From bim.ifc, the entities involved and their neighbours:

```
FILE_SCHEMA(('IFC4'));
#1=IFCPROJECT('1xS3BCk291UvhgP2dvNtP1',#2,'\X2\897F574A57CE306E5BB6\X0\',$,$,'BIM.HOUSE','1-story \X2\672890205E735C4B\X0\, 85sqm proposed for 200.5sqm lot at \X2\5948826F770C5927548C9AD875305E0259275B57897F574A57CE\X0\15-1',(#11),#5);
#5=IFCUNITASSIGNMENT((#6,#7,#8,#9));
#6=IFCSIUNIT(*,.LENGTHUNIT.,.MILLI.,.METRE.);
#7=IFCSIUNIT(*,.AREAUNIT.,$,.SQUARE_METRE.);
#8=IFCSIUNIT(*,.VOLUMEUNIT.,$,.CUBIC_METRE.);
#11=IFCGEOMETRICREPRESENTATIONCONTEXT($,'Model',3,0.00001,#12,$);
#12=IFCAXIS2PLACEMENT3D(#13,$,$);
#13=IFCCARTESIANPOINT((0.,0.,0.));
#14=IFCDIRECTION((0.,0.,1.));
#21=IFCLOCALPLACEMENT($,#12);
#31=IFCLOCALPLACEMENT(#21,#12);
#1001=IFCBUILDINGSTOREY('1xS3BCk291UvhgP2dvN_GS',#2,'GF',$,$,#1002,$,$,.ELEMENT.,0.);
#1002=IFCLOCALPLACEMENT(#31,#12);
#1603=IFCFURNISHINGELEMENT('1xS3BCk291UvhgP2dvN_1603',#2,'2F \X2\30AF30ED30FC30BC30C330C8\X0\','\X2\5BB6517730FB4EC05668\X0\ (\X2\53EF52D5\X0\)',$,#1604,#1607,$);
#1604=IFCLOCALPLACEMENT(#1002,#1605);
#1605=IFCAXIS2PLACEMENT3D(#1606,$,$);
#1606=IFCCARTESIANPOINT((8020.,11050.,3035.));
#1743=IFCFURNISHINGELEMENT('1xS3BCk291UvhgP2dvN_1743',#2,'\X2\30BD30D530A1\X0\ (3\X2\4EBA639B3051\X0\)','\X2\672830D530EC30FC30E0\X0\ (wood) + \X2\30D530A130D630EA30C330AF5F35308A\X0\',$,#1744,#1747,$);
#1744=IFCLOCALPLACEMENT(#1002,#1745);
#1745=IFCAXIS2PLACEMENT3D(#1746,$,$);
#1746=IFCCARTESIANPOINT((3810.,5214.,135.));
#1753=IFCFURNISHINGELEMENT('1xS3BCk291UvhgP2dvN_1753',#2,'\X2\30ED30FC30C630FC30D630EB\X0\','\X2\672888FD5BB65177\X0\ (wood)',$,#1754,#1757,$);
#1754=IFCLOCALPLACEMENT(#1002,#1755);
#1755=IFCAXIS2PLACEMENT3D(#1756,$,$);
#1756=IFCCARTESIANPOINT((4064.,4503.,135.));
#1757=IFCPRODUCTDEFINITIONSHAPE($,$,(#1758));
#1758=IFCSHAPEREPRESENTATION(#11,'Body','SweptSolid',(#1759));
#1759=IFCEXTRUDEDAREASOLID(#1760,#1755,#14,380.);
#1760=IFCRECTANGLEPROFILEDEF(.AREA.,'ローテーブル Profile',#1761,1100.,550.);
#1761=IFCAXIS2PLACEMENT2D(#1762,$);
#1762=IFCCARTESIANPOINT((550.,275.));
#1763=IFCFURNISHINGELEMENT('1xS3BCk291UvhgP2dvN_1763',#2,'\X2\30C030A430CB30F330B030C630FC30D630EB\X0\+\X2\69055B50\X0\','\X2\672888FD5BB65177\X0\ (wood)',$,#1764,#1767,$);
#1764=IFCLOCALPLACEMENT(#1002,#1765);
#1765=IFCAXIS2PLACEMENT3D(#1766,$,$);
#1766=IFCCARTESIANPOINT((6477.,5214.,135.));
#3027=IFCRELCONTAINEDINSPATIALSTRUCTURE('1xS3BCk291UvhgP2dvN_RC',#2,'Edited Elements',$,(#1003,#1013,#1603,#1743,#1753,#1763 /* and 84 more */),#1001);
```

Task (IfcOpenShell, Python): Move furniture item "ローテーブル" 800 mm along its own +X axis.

```python
import ifcopenshell
import ifcopenshell.api.geometry
import ifcopenshell.util.placement
import ifcopenshell.util.unit

model = ifcopenshell.open("bim.ifc")
unit_scale = ifcopenshell.util.unit.calculate_unit_scale(model)

item = model.by_id(1753)
matrix = ifcopenshell.util.placement.get_local_placement(item.ObjectPlacement)
matrix[:3, 3] += matrix[:3, 0] * 0.8 / unit_scale
ifcopenshell.api.geometry.edit_object_placement(model, product=item, matrix=matrix, is_si=False)

print(ifcopenshell.util.placement.get_local_placement(item.ObjectPlacement).round(3) + 0.0)

model.write("bim-out.ifc")
```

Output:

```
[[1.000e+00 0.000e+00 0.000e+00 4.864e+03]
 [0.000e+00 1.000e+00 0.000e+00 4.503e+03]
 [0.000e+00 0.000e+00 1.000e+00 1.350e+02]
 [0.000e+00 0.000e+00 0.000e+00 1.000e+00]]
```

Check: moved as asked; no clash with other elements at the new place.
